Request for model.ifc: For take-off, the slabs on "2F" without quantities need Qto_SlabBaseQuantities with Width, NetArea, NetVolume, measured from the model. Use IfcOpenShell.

First a look at what the model holds.

```python
import ifcopenshell
import ifcopenshell.util.element
import ifcopenshell.util.unit

model = ifcopenshell.open("model.ifc")
print(model.schema)
for unit_type in ("LENGTHUNIT", "AREAUNIT", "VOLUMEUNIT"):
    print(unit_type, ifcopenshell.util.unit.calculate_unit_scale(model, unit_type))
storey = next(s for s in model.by_type("IfcBuildingStorey") if s.Name == "2F")
slabs = [e for e in ifcopenshell.util.element.get_decomposition(storey) if e.is_a("IfcSlab")]
for e in sorted(slabs, key=lambda e: e.id()):
    print(e.id(), e.is_a(), e.Name, list(ifcopenshell.util.element.get_psets(e, qtos_only=True)), sep=" | ")
```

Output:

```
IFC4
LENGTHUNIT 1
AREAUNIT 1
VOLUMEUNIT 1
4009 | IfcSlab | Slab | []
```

```python
import ifcopenshell
import ifcopenshell.api.pset
import ifcopenshell.geom
import ifcopenshell.util.element
import ifcopenshell.util.shape
import ifcopenshell.util.unit

model = ifcopenshell.open("model.ifc")
unit_scale = ifcopenshell.util.unit.calculate_unit_scale(model)
area_scale = ifcopenshell.util.unit.calculate_unit_scale(model, "AREAUNIT")
volume_scale = ifcopenshell.util.unit.calculate_unit_scale(model, "VOLUMEUNIT")
settings = ifcopenshell.geom.settings()

storey = next(s for s in model.by_type("IfcBuildingStorey") if s.Name == "2F")
slabs = [e for e in ifcopenshell.util.element.get_decomposition(storey) if e.is_a("IfcSlab")]

for e in sorted(slabs, key=lambda e: e.id()):
    if ifcopenshell.util.element.get_psets(e, qtos_only=True, should_inherit=False):
        continue
    # Geometry comes back in metres, in the element's own axes.
    shape = ifcopenshell.geom.create_shape(settings, e)
    values = {
        "Width": ifcopenshell.util.shape.get_z(shape.geometry) / unit_scale,
        "NetArea": ifcopenshell.util.shape.get_footprint_area(shape.geometry) / area_scale,
        "NetVolume": ifcopenshell.util.shape.get_volume(shape.geometry) / volume_scale,
    }
    qto = ifcopenshell.api.pset.add_qto(model, product=e, name="Qto_SlabBaseQuantities")
    ifcopenshell.api.pset.edit_qto(model, qto=qto, properties=values)
    print(e.id(), {k: round(v, 3) for k, v in values.items()})

model.write("model_rev.ifc")
```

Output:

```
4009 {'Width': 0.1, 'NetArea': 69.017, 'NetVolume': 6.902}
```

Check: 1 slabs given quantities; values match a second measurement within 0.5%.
